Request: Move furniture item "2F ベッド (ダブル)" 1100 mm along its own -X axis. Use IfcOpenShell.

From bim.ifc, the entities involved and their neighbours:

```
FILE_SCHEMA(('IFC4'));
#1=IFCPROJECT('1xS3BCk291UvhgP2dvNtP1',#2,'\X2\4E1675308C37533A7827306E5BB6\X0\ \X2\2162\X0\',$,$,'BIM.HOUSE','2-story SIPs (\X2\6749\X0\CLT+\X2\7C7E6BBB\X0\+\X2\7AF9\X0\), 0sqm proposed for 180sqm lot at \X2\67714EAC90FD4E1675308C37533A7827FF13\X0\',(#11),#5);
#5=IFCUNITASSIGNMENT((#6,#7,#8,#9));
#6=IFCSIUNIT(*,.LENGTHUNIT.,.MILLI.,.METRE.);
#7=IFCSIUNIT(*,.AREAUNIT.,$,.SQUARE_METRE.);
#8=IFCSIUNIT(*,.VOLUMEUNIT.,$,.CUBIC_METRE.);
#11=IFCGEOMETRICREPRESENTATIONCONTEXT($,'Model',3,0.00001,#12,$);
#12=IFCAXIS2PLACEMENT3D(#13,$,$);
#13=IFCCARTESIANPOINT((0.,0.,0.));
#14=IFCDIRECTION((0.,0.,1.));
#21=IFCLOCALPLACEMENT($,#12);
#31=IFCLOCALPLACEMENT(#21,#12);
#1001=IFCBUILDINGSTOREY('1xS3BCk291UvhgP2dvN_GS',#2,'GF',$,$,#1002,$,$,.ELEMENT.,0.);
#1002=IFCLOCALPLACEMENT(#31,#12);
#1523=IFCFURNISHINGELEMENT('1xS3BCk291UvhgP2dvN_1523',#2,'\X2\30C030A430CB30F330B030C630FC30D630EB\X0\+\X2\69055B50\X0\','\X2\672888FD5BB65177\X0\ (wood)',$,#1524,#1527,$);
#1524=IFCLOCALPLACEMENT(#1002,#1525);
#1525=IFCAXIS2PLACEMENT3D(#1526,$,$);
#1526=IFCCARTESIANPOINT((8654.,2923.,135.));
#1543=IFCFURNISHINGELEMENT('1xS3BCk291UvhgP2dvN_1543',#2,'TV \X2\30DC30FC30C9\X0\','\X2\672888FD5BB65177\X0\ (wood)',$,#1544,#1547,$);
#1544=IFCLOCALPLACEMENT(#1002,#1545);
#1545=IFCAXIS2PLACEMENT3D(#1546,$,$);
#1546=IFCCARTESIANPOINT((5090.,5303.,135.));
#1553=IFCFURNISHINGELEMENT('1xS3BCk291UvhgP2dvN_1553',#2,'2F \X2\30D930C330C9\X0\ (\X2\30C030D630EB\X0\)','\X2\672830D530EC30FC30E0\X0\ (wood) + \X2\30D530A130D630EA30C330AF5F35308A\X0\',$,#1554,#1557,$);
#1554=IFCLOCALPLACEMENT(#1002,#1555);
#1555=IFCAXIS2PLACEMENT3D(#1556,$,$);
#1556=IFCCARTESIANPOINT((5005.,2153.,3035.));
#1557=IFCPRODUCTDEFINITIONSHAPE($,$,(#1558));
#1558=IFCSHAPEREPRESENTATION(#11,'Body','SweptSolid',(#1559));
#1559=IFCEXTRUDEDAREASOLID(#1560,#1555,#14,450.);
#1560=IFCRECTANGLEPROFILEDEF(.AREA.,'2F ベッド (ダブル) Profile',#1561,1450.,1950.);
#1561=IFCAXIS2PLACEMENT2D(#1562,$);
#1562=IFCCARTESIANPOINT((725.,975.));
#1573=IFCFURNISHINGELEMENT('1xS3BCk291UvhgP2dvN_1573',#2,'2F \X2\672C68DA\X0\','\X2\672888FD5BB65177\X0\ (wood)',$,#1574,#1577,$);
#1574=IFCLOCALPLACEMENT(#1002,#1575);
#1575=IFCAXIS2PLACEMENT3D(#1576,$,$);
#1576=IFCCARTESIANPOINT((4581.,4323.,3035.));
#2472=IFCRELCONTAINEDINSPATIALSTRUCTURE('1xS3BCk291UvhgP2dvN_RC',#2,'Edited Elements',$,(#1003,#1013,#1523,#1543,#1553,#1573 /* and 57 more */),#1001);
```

```python
import ifcopenshell
import ifcopenshell.api.geometry
import ifcopenshell.util.placement

model = ifcopenshell.open("bim.ifc")

item = model.by_guid("1xS3BCk291UvhgP2dvN_1553")
matrix = ifcopenshell.util.placement.get_local_placement(item.ObjectPlacement)
matrix[:3, 3] -= matrix[:3, 0] * 1100.0
ifcopenshell.api.geometry.edit_object_placement(model, product=item, matrix=matrix, is_si=False)

print(ifcopenshell.util.placement.get_local_placement(item.ObjectPlacement).round(3) + 0.0)

model.write("bim_rev.ifc")
```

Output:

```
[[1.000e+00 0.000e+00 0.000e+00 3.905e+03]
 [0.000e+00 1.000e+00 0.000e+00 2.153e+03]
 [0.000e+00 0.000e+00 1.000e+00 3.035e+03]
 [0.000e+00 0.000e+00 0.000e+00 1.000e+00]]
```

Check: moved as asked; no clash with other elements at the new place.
